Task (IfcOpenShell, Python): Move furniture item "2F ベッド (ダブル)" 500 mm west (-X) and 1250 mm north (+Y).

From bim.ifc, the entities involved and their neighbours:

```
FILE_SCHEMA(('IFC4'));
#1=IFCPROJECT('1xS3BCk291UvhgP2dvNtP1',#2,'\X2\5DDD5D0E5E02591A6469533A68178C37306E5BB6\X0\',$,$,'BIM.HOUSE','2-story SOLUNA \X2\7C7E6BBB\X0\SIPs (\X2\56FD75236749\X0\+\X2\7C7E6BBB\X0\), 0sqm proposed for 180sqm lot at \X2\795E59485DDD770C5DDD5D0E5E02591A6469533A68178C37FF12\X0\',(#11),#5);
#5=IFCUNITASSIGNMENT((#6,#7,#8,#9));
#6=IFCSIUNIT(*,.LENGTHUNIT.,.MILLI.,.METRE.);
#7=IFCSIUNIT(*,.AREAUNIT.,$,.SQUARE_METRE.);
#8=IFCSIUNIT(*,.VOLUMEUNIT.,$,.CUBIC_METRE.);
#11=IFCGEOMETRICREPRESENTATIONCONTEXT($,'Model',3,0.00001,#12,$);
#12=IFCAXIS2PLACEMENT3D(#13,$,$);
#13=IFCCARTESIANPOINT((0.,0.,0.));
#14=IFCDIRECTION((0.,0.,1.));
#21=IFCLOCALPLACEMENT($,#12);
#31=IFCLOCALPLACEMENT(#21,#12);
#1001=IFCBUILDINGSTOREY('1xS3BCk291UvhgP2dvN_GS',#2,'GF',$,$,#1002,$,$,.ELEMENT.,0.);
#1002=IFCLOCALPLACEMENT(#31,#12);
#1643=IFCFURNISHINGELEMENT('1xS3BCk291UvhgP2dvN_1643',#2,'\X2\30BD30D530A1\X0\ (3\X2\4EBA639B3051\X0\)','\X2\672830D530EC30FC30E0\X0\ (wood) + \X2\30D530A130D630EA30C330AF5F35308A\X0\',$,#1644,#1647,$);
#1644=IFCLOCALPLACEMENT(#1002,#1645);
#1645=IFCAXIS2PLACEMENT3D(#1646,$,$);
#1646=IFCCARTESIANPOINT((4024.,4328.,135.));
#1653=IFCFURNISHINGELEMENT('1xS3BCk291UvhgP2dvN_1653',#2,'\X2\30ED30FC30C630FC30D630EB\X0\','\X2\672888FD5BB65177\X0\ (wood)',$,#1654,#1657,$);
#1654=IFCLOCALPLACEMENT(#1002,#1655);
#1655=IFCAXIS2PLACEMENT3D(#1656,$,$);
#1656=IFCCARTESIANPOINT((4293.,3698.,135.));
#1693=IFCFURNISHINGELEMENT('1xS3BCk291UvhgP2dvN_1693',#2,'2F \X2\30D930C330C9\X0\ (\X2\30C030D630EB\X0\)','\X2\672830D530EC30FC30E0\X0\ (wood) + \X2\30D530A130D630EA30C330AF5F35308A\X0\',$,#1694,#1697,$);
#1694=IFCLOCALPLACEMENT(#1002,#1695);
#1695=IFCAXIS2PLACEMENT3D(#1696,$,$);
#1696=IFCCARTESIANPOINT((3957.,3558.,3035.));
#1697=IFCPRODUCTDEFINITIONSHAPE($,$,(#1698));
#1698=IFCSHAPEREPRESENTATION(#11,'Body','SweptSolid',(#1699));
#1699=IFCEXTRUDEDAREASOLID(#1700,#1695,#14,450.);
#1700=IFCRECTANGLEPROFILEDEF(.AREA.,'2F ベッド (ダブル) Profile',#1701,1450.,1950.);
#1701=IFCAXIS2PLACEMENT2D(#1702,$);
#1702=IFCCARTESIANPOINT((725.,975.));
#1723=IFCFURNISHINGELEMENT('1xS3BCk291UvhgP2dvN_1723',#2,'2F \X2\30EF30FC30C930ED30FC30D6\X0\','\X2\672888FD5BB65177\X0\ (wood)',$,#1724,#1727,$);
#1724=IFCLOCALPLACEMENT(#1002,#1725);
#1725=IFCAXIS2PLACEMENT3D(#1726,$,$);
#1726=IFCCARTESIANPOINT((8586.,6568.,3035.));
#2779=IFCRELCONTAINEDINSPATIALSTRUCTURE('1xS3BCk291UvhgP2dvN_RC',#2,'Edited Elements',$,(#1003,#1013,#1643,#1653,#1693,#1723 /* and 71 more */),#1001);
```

```python
import ifcopenshell
import ifcopenshell.api.geometry
import ifcopenshell.util.placement
import ifcopenshell.util.unit

model = ifcopenshell.open("bim.ifc")
unit_scale = ifcopenshell.util.unit.calculate_unit_scale(model)

item = model.by_guid("1xS3BCk291UvhgP2dvN_1693")
matrix = ifcopenshell.util.placement.get_local_placement(item.ObjectPlacement)
matrix[0, 3] -= 0.5 / unit_scale
matrix[1, 3] += 1.25 / unit_scale
ifcopenshell.api.geometry.edit_object_placement(model, product=item, matrix=matrix, is_si=False)

print(ifcopenshell.util.placement.get_local_placement(item.ObjectPlacement).round(3) + 0.0)

model.write("bim_updated.ifc")
```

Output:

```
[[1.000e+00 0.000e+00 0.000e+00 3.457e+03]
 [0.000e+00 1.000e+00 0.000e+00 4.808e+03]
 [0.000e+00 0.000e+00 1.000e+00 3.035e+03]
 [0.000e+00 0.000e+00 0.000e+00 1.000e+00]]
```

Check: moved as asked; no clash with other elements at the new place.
